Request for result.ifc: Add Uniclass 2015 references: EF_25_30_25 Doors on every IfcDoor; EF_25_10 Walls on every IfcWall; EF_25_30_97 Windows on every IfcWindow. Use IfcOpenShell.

First a look at what the model holds.

```python
import ifcopenshell

model = ifcopenshell.open("result.ifc")
print(model.schema)
print("classifications:", [c.Name for c in model.by_type("IfcClassification")])
for ifc_class in ("IfcDoor", "IfcRoof", "IfcStair", "IfcWall", "IfcWindow"):
    print(ifc_class, len(model.by_type(ifc_class)))
```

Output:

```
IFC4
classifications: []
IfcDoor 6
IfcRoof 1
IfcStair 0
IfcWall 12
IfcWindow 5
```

```python
import ifcopenshell
import ifcopenshell.api.classification

model = ifcopenshell.open("result.ifc")

system = ifcopenshell.api.classification.add_classification(model, classification="Uniclass 2015")

codes = {
    "IfcDoor": ("EF_25_30_25", "Doors"),
    "IfcWall": ("EF_25_10", "Walls"),
    "IfcWindow": ("EF_25_30_97", "Windows"),
}
for ifc_class, (code, name) in codes.items():
    products = model.by_type(ifc_class)
    ifcopenshell.api.classification.add_reference(
        model, products=products, classification=system, identification=code, name=name
    )
    print(code, len(products))

model.write("result_v2.ifc")
```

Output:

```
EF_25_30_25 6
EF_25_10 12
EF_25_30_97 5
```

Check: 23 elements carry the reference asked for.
